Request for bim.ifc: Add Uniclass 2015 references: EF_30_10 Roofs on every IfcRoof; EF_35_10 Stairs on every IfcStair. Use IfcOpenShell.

First a look at what the model holds.

```python
import ifcopenshell

model = ifcopenshell.open("bim.ifc")
print(model.schema)
print("classifications:", [c.Name for c in model.by_type("IfcClassification")])
for ifc_class in ("IfcDoor", "IfcRoof", "IfcStair", "IfcWall", "IfcWindow"):
    print(ifc_class, len(model.by_type(ifc_class)))
```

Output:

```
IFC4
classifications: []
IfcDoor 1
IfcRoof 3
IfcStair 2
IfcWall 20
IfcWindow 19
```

```python
import ifcopenshell
import ifcopenshell.api.classification

model = ifcopenshell.open("bim.ifc")

system = ifcopenshell.api.classification.add_classification(model, classification="Uniclass 2015")

codes = {
    "IfcRoof": ("EF_30_10", "Roofs"),
    "IfcStair": ("EF_35_10", "Stairs"),
}
for ifc_class, (code, name) in codes.items():
    products = model.by_type(ifc_class)
    ifcopenshell.api.classification.add_reference(
        model, products=products, classification=system, identification=code, name=name
    )
    print(code, len(products))

model.write("bim-out.ifc")
```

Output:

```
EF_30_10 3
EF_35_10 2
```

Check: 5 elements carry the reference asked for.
